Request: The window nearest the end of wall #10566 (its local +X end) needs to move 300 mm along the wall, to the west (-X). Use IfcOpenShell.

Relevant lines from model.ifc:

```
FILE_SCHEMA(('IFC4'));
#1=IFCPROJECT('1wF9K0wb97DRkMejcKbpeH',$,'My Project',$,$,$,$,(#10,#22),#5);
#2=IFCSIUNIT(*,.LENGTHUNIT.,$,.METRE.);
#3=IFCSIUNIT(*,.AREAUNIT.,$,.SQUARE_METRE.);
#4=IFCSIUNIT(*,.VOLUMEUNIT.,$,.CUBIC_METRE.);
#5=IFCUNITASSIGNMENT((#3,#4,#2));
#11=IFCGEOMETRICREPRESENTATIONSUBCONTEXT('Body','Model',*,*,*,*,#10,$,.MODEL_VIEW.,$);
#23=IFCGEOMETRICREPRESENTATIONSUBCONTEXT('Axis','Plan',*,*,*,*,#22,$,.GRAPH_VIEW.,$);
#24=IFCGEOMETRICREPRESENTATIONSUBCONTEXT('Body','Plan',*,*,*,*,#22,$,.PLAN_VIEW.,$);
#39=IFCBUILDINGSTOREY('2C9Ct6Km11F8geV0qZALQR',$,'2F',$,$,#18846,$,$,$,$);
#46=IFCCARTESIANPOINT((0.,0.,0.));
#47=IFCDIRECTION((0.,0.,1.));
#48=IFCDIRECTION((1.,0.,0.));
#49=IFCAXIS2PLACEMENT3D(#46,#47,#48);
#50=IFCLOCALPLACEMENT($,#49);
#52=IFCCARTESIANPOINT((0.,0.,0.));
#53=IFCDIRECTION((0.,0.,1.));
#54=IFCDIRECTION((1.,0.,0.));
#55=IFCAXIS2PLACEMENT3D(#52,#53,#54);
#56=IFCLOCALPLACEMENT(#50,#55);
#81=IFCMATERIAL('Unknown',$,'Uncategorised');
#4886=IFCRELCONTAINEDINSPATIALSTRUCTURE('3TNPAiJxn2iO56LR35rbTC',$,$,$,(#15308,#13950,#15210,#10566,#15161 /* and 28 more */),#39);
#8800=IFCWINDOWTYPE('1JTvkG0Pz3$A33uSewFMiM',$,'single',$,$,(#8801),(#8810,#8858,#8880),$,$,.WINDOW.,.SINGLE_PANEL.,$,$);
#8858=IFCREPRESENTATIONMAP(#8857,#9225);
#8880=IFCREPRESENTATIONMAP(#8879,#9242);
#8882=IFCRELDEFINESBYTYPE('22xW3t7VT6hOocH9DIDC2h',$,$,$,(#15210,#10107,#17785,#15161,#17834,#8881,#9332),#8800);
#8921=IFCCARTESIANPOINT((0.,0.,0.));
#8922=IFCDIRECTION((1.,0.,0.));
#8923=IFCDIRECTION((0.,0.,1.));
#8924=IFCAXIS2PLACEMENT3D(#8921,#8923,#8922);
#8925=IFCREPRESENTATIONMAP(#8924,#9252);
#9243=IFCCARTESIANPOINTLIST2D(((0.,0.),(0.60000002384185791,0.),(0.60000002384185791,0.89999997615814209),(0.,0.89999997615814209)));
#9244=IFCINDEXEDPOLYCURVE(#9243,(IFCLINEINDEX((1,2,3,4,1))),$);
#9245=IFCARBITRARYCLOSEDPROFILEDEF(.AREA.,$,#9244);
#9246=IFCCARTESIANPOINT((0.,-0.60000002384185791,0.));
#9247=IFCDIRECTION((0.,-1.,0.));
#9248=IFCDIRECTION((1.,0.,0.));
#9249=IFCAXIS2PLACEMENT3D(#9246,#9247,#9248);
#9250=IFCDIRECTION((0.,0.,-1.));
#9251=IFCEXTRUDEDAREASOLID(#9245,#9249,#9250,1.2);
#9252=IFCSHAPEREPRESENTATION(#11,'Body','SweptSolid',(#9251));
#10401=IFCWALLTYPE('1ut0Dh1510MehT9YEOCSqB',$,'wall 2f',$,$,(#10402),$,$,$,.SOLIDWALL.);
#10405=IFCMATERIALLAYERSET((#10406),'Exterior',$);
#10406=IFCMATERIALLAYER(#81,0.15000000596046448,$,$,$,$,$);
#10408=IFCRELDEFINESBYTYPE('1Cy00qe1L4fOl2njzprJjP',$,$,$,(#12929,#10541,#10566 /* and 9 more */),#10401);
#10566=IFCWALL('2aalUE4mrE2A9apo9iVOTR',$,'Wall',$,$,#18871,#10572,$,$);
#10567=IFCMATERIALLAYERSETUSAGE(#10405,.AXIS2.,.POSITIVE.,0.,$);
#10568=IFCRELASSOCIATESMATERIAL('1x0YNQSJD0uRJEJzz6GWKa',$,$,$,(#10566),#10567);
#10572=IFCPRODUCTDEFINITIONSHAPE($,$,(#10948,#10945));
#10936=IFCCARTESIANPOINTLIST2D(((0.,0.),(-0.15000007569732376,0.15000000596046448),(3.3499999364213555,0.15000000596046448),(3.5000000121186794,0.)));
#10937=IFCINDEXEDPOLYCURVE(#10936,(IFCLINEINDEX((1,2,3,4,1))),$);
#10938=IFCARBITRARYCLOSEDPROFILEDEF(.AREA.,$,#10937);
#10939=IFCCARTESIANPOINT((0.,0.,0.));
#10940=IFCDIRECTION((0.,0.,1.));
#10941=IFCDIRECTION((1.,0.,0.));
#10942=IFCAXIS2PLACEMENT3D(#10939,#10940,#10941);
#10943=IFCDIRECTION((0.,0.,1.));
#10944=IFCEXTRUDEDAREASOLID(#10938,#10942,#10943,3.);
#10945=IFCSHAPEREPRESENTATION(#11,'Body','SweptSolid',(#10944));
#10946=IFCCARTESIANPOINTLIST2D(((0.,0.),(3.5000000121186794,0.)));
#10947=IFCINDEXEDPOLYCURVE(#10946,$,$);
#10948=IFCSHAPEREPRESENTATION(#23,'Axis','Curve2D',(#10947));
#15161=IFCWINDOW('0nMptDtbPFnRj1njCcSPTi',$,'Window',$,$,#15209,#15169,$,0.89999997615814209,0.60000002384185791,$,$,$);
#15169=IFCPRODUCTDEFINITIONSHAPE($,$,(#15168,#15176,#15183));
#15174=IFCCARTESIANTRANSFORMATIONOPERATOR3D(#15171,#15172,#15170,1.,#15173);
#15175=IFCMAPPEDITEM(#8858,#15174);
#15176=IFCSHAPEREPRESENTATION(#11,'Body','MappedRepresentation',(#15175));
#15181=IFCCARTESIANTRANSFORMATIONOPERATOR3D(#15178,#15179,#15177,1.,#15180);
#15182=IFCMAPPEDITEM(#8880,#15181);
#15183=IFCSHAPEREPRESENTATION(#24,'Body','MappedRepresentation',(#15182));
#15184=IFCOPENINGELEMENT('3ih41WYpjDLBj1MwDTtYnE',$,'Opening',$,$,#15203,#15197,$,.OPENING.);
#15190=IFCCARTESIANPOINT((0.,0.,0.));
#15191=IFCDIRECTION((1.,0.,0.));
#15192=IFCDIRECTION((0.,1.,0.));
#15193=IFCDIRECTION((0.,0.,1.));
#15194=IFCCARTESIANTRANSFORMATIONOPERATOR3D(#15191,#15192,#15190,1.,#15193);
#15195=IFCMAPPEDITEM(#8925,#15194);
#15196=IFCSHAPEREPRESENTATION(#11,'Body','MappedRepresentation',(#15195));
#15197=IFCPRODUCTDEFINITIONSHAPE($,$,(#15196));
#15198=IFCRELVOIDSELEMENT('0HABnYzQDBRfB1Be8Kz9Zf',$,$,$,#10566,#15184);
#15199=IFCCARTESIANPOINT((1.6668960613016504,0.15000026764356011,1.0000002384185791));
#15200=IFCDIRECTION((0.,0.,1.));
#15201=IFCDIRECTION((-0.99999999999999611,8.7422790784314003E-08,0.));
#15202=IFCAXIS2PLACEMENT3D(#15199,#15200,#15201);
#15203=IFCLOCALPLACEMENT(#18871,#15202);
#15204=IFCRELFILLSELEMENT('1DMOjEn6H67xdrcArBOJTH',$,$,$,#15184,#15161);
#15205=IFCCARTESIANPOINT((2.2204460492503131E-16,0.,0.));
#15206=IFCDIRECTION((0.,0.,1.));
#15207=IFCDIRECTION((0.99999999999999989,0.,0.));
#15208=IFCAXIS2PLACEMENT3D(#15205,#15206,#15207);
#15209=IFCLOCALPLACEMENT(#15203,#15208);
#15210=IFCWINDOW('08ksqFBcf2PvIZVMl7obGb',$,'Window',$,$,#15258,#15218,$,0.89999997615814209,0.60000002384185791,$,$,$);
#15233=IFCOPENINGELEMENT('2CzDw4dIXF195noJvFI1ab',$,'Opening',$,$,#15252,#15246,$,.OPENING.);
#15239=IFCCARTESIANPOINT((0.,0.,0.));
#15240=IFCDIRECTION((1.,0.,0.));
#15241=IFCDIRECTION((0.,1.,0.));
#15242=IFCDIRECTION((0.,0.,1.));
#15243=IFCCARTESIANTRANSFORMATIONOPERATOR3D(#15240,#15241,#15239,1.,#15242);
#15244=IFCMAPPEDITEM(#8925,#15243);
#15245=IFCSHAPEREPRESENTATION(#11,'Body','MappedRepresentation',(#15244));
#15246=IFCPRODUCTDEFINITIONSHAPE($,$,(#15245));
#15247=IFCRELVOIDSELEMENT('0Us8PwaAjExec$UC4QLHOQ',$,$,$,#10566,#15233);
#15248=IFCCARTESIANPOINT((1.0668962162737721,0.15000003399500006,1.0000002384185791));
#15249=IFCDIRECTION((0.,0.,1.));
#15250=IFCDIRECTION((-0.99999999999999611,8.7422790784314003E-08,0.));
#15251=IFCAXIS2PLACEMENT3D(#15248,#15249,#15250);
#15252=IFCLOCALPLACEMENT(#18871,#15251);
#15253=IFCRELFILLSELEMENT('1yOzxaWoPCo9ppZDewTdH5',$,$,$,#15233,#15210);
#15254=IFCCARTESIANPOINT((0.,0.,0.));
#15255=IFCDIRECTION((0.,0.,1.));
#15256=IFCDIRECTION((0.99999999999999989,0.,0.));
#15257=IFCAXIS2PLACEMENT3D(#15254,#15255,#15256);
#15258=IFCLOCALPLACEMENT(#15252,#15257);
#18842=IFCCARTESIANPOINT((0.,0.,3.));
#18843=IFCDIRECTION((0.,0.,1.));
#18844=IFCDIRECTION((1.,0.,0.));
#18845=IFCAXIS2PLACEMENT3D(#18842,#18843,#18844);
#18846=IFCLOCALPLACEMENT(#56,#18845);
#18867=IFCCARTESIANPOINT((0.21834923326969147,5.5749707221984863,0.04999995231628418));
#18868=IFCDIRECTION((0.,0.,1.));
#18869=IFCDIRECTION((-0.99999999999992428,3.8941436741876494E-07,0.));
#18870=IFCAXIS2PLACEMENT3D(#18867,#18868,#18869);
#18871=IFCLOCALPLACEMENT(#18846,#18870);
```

```python
import ifcopenshell
import ifcopenshell.api.geometry
import ifcopenshell.util.placement

model = ifcopenshell.open("model.ifc")

window = model.by_id(15161)
opening = window.FillsVoids[0].RelatingOpeningElement
wall = opening.VoidsElements[0].RelatingBuildingElement

wall_matrix = ifcopenshell.util.placement.get_local_placement(wall.ObjectPlacement)
shift = wall_matrix[:3, 0] * 0.3
before = ifcopenshell.util.placement.get_local_placement(window.ObjectPlacement)[:3, 3].copy()

# The window is placed relative to its opening, so it follows when the opening moves.
matrix = ifcopenshell.util.placement.get_local_placement(opening.ObjectPlacement)
matrix[:3, 3] += shift
ifcopenshell.api.geometry.edit_object_placement(
    model, product=opening, matrix=matrix, is_si=False, should_transform_children=True
)

after = ifcopenshell.util.placement.get_local_placement(window.ObjectPlacement)[:3, 3]
print("window moved by", (after - before).round(3) + 0.0)

model.write("model_updated.ifc")
```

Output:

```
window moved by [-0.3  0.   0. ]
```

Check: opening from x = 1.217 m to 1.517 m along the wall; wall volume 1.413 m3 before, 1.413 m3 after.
